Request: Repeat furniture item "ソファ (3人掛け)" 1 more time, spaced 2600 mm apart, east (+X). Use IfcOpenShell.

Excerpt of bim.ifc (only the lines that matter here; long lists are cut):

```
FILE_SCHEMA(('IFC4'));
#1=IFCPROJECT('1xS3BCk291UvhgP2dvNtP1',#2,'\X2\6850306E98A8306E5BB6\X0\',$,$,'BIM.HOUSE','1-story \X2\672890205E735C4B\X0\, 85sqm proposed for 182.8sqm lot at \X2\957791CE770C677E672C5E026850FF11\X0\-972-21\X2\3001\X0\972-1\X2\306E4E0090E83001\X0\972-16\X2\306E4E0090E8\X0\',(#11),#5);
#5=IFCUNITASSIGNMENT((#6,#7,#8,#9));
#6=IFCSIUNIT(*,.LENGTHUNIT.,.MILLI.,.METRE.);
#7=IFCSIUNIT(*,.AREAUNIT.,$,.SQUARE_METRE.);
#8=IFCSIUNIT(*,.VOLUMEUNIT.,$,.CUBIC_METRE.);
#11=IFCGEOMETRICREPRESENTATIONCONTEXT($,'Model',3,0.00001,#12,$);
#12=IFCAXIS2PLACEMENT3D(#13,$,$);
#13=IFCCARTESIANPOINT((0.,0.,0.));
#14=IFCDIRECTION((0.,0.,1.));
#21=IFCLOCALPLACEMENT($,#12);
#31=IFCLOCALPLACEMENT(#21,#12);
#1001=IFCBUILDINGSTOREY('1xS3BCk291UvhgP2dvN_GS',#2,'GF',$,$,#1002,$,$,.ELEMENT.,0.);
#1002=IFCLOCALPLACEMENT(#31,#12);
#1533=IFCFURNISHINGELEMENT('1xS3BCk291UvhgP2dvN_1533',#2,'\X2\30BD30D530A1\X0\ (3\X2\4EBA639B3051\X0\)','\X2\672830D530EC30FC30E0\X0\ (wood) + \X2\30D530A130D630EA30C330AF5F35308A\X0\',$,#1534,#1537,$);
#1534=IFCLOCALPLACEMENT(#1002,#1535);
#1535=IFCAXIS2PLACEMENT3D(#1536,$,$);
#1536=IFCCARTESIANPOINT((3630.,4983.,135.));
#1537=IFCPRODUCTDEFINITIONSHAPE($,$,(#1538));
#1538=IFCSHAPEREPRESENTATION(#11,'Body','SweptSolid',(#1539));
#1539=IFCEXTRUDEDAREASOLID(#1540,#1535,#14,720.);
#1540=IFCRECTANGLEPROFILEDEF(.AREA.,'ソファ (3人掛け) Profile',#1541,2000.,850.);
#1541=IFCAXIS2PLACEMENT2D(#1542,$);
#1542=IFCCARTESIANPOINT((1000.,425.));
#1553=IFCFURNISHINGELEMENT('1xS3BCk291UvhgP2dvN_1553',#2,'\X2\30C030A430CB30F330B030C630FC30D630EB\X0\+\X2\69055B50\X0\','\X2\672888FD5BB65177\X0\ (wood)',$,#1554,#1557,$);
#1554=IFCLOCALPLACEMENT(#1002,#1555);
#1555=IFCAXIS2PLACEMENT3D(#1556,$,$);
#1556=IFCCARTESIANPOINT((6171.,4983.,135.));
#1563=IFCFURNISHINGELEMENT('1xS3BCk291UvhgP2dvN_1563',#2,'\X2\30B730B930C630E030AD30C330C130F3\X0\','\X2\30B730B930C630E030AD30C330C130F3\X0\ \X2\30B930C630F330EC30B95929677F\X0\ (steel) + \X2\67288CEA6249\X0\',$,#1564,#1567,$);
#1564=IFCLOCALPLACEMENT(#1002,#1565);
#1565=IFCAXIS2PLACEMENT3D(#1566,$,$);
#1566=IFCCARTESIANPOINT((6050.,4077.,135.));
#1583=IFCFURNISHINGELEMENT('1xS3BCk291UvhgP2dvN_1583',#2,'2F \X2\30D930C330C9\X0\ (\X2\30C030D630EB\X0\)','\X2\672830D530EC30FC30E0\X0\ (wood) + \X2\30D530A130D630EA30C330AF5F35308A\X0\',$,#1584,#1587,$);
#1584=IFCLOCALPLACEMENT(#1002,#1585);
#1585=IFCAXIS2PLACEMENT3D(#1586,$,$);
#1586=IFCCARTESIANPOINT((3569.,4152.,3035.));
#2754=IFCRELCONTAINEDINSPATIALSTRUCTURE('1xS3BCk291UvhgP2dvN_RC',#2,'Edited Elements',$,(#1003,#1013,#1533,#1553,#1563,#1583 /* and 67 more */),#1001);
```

```python
import numpy as np
import ifcopenshell
import ifcopenshell.api.geometry
import ifcopenshell.api.root
import ifcopenshell.util.element
import ifcopenshell.util.placement
import ifcopenshell.util.unit

model = ifcopenshell.open("bim.ifc")
unit_scale = ifcopenshell.util.unit.calculate_unit_scale(model)


def reuse_history(source, copy):
    """copy_class also copies each property set's owner history, people and application; keep the originals."""
    for rel in copy.IsDefinedBy:
        if rel.is_a("IfcRelDefinesByProperties") and (history := rel.RelatingPropertyDefinition.OwnerHistory):
            rel.RelatingPropertyDefinition.OwnerHistory = source.OwnerHistory
            ifcopenshell.util.element.remove_deep2(model, history)


source = model.by_id(1533)
base = ifcopenshell.util.placement.get_local_placement(source.ObjectPlacement)
step = np.array([1.0, 0.0, 0.0]) * 2.6 / unit_scale

for i in range(1, 2):
    copy = ifcopenshell.api.root.copy_class(model, product=source)
    copy.Representation = ifcopenshell.util.element.copy_deep(
        model, source.Representation, exclude=["IfcGeometricRepresentationContext", "IfcRepresentationMap"]
    )
    reuse_history(source, copy)
    matrix = base.copy()
    matrix[:3, 3] += i * step
    print("added at", matrix[:3, 3].round(3) + 0.0)
    ifcopenshell.api.geometry.edit_object_placement(model, product=copy, matrix=matrix, is_si=False)

model.write("bim_edited.ifc")
```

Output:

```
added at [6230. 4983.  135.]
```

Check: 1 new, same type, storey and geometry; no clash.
